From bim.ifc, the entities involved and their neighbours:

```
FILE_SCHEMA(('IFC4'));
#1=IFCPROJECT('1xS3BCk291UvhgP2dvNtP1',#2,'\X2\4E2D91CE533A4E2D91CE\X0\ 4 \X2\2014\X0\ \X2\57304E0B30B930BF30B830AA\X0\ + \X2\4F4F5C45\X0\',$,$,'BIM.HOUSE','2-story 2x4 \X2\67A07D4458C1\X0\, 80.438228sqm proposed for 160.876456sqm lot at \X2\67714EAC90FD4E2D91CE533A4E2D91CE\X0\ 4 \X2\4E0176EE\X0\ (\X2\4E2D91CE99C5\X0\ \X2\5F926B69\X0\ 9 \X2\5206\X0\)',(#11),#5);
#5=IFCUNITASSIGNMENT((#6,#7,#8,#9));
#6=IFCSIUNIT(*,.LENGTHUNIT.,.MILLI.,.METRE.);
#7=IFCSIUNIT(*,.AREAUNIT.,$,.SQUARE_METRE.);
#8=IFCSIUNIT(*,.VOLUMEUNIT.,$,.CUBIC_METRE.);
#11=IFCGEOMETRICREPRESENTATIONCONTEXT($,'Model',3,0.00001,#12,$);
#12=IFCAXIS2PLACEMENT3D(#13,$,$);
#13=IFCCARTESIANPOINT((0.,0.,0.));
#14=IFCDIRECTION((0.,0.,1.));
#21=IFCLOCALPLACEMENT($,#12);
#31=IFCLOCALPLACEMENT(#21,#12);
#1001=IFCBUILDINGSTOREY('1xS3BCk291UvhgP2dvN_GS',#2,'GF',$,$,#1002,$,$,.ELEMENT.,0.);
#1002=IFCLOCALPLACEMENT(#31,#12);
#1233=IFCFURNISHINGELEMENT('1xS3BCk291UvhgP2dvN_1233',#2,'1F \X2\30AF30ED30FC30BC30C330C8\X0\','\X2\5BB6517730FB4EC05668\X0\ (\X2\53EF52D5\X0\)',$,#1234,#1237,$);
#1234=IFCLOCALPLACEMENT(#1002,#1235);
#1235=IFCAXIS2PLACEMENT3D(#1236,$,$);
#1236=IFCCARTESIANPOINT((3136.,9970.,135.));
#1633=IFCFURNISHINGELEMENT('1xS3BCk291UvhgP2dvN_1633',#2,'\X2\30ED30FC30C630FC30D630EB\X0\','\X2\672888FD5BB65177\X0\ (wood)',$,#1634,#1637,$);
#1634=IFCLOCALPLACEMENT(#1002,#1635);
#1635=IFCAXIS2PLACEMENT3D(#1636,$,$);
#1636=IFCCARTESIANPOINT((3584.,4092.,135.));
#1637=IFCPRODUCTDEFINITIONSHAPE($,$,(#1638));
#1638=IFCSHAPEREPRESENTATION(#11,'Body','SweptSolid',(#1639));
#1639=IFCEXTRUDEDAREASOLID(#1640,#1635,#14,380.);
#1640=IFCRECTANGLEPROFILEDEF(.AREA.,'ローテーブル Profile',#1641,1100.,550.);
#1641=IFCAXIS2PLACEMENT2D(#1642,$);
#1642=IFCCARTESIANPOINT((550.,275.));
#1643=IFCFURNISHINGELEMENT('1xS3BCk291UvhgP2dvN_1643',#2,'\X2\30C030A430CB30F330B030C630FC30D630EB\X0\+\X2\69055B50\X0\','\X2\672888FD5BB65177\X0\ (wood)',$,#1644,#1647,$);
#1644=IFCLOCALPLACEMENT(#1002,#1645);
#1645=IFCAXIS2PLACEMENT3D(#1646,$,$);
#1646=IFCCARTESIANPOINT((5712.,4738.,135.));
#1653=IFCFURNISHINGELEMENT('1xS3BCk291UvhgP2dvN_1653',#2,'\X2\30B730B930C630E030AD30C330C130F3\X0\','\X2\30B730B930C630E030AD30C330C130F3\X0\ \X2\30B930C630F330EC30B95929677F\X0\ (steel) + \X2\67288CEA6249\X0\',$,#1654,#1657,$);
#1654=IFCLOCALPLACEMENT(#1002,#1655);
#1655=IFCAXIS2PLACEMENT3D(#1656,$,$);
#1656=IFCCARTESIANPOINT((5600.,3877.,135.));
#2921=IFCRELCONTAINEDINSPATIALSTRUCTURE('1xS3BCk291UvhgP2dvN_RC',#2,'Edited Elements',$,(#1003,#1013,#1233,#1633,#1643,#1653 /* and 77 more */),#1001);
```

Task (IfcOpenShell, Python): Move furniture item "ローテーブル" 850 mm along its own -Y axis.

```python
import ifcopenshell
import ifcopenshell.api.geometry
import ifcopenshell.util.placement

model = ifcopenshell.open("bim.ifc")

item = model.by_id(1633)
matrix = ifcopenshell.util.placement.get_local_placement(item.ObjectPlacement)
matrix[:3, 3] -= matrix[:3, 1] * 850.0
ifcopenshell.api.geometry.edit_object_placement(model, product=item, matrix=matrix, is_si=False)

print(ifcopenshell.util.placement.get_local_placement(item.ObjectPlacement).round(3) + 0.0)

model.write("bim_edited.ifc")
```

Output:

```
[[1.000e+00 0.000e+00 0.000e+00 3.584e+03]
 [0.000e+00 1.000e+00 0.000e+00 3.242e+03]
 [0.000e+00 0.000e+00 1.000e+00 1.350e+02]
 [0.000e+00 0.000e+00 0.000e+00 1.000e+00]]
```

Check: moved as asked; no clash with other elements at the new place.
